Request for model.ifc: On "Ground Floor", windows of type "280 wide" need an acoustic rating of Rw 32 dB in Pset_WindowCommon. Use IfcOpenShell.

First a look at what the model holds.

```python
import ifcopenshell
import ifcopenshell.util.element

model = ifcopenshell.open("model.ifc")
print(model.schema)
storey = next(s for s in model.by_type("IfcBuildingStorey") if s.Name == "Ground Floor")
windows = [e for e in ifcopenshell.util.element.get_decomposition(storey) if e.is_a("IfcWindow")]
seen = {}
for e in windows:
    element_type = ifcopenshell.util.element.get_type(e)
    key = (element_type.Name if element_type != e and element_type else None, ifcopenshell.util.element.get_pset(e, "Pset_WindowCommon", "AcousticRating"))
    seen[key] = seen.get(key, 0) + 1
for (name, value), count in sorted(seen.items(), key=str):
    print(count, "x", name, "|", value)
```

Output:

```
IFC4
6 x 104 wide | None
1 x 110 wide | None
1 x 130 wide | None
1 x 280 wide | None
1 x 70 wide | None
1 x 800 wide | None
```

```python
import ifcopenshell
import ifcopenshell.api.pset
import ifcopenshell.util.element

model = ifcopenshell.open("model.ifc")

storey = next(s for s in model.by_type("IfcBuildingStorey") if s.Name == "Ground Floor")
windows = [e for e in ifcopenshell.util.element.get_decomposition(storey) if e.is_a("IfcWindow")]

count = 0
for e in windows:
    element_type = ifcopenshell.util.element.get_type(e)
    if element_type in (None, e) or element_type.Name != "280 wide":
        continue
    # add_pset returns the element's existing set when there is one.
    pset = ifcopenshell.api.pset.add_pset(model, product=e, name="Pset_WindowCommon")
    ifcopenshell.api.pset.edit_pset(model, pset=pset, properties={"AcousticRating": "Rw 32 dB"})
    count += 1

print(count, "windows updated")

model.write("model_updated.ifc")
```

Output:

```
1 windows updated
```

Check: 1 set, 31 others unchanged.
